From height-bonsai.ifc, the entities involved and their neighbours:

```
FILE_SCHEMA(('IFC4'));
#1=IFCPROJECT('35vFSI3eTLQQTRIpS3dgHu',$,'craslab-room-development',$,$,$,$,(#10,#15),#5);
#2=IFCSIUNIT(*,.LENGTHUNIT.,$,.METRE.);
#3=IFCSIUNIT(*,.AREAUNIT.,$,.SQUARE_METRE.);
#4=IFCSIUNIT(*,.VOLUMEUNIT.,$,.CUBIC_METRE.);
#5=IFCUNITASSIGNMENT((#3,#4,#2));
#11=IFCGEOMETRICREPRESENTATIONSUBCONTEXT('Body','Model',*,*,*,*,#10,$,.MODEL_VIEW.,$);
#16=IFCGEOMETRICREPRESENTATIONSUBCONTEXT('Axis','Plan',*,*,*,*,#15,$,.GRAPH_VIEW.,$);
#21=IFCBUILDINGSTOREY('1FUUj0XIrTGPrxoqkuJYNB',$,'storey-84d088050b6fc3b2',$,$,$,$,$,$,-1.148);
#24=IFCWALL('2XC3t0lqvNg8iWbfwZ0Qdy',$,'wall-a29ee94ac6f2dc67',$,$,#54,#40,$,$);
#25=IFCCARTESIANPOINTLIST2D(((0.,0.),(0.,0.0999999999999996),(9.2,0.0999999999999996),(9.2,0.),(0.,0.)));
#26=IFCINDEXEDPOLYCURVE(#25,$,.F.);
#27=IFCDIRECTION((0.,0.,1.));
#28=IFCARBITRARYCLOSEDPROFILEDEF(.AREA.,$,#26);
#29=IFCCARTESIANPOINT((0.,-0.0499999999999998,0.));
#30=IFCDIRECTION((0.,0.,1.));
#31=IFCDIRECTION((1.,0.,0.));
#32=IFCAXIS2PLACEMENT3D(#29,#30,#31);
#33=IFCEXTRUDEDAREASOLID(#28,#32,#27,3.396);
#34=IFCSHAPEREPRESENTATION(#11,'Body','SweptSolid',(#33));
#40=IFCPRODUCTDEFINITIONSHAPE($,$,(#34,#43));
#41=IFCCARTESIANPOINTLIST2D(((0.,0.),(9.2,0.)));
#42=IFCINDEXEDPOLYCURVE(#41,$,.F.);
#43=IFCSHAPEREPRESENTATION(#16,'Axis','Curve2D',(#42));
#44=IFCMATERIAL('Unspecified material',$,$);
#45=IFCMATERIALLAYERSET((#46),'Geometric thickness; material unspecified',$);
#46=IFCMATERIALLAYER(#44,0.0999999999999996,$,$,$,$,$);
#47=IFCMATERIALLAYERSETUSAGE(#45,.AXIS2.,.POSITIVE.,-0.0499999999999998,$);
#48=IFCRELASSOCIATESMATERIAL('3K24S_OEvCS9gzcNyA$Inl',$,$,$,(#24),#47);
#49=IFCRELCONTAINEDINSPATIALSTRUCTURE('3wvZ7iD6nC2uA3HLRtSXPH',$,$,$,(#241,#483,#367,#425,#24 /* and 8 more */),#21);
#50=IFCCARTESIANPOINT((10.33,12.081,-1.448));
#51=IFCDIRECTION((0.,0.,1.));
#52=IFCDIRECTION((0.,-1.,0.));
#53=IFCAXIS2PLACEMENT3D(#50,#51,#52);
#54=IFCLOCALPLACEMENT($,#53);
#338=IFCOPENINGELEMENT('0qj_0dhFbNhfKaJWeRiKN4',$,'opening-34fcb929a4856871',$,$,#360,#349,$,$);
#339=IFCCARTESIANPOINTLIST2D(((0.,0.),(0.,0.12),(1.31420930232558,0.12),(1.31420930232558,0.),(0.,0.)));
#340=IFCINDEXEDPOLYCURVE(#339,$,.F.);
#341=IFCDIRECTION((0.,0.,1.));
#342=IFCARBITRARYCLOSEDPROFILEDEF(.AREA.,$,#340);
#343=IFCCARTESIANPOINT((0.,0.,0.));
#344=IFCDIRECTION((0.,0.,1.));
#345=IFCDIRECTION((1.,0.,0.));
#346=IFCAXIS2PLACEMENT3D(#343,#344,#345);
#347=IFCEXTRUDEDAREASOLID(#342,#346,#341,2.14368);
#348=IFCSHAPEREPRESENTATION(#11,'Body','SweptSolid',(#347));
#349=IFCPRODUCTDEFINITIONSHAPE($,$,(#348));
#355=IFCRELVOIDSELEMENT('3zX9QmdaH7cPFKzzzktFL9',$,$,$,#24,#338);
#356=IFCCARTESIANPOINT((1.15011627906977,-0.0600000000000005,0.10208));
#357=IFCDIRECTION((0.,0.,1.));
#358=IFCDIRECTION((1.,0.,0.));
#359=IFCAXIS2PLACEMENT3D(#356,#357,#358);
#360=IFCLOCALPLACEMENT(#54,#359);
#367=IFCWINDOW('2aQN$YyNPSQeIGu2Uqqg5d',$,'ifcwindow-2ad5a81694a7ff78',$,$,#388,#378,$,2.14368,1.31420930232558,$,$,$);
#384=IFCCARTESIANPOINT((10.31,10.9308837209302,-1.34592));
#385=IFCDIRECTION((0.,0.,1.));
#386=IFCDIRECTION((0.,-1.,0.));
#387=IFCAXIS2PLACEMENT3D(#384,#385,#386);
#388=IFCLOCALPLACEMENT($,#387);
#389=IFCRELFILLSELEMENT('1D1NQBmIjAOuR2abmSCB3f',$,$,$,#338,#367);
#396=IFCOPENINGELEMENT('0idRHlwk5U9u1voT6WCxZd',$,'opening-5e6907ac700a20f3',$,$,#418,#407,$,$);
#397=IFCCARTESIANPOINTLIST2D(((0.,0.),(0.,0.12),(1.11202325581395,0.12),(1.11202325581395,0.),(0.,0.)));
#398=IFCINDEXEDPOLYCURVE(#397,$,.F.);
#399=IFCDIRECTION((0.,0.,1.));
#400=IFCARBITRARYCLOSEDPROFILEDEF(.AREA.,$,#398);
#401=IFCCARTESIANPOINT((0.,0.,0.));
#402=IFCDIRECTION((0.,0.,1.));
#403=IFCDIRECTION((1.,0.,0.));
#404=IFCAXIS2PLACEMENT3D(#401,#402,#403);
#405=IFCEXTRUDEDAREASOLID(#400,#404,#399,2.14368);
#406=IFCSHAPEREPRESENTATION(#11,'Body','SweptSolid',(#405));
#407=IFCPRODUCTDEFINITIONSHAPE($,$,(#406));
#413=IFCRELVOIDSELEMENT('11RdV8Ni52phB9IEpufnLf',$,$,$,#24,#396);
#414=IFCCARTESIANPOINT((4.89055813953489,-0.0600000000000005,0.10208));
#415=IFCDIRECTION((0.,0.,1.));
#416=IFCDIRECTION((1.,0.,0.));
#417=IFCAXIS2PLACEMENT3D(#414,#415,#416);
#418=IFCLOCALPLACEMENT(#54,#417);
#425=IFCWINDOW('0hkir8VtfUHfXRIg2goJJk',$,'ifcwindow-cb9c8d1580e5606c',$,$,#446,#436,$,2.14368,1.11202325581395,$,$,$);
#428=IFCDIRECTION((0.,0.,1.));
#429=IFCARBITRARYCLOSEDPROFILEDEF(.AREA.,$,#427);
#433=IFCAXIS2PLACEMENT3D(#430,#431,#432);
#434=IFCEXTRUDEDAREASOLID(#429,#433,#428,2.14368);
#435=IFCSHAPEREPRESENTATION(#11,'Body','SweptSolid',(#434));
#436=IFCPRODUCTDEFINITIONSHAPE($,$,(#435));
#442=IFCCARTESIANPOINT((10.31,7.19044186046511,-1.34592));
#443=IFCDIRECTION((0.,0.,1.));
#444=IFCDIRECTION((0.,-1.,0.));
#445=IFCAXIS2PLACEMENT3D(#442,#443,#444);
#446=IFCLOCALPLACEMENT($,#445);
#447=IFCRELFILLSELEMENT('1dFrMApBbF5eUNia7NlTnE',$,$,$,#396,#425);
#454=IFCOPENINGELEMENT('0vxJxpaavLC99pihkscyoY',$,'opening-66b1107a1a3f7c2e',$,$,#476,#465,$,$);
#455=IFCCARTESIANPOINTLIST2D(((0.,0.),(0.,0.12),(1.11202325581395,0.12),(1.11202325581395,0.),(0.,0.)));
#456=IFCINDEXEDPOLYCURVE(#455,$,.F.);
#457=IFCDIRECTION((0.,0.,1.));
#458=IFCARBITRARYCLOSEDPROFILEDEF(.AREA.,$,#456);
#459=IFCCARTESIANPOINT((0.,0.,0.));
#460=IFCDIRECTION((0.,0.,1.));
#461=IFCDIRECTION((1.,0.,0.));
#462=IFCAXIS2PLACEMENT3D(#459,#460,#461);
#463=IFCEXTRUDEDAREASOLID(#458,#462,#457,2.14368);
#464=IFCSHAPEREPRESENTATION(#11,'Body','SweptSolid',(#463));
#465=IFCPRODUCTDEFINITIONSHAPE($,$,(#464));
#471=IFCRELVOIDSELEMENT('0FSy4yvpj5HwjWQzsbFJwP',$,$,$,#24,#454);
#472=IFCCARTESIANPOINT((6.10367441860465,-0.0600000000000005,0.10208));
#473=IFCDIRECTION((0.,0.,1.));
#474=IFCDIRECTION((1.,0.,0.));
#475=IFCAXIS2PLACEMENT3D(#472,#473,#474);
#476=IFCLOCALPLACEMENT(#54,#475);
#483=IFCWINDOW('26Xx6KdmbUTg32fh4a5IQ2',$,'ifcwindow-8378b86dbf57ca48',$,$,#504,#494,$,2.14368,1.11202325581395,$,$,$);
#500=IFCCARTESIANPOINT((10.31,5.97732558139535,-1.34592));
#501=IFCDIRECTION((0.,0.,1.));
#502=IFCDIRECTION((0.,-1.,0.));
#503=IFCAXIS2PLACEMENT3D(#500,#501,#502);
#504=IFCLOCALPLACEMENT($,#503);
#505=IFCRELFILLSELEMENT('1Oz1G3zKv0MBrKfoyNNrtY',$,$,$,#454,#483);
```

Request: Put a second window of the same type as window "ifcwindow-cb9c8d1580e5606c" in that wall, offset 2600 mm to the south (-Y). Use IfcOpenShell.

```python
import ifcopenshell
import ifcopenshell.api.feature
import ifcopenshell.api.geometry
import ifcopenshell.api.root
import ifcopenshell.geom
import ifcopenshell.util.element
import ifcopenshell.util.placement
import ifcopenshell.util.shape

model = ifcopenshell.open("height-bonsai.ifc")
settings = ifcopenshell.geom.settings()


def volume(element):
    """Net volume in cubic metres, openings subtracted."""
    shape = ifcopenshell.geom.create_shape(settings, element)
    return ifcopenshell.util.shape.get_volume(shape.geometry)


window = model.by_guid("0hkir8VtfUHfXRIg2goJJk")
opening = window.FillsVoids[0].RelatingOpeningElement
wall = opening.VoidsElements[0].RelatingBuildingElement
before = volume(wall)
shift = ifcopenshell.util.placement.get_local_placement(wall.ObjectPlacement)[:3, 0] * 2.6

# copy_class copies the void relationship, type, container and properties, but no geometry.
new_opening = ifcopenshell.api.root.copy_class(model, product=opening)
new_opening.Representation = ifcopenshell.util.element.copy_deep(
    model, opening.Representation, exclude=["IfcGeometricRepresentationContext", "IfcRepresentationMap"]
)
new_window = ifcopenshell.api.root.copy_class(model, product=window)
new_window.Representation = ifcopenshell.util.element.copy_deep(
    model, window.Representation, exclude=["IfcGeometricRepresentationContext", "IfcRepresentationMap"]
)
ifcopenshell.api.feature.add_filling(model, opening=new_opening, element=new_window)

for old, new in ((opening, new_opening), (window, new_window)):
    matrix = ifcopenshell.util.placement.get_local_placement(old.ObjectPlacement)
    matrix[:3, 3] += shift
    ifcopenshell.api.geometry.edit_object_placement(model, product=new, matrix=matrix, is_si=False)

after = volume(wall)

print(f"wall volume {before:.3f} -> {after:.3f} m3")

model.write("height-bonsai_updated.ifc")
```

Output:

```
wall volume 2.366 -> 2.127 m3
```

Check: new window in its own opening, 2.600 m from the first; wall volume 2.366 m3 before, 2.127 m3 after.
